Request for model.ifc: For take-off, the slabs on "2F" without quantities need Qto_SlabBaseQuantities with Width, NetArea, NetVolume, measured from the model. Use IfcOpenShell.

First a look at what the model holds.

```python
import ifcopenshell
import ifcopenshell.util.element
import ifcopenshell.util.unit

model = ifcopenshell.open("model.ifc")
print(model.schema)
for unit_type in ("LENGTHUNIT", "AREAUNIT", "VOLUMEUNIT"):
    print(unit_type, ifcopenshell.util.unit.calculate_unit_scale(model, unit_type))
storey = next(s for s in model.by_type("IfcBuildingStorey") if s.Name == "2F")
slabs = [e for e in ifcopenshell.util.element.get_decomposition(storey) if e.is_a("IfcSlab")]
for e in sorted(slabs, key=lambda e: e.id()):
    print(e.id(), e.is_a(), e.Name, list(ifcopenshell.util.element.get_psets(e, qtos_only=True)), sep=" | ")
```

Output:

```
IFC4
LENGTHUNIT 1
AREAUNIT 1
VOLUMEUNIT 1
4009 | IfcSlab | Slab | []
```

```python
import ifcopenshell
import ifcopenshell.api.pset
import ifcopenshell.geom
import ifcopenshell.util.element
import ifcopenshell.util.shape
import ifcopenshell.util.unit

model = ifcopenshell.open("model.ifc")
unit_scale = ifcopenshell.util.unit.calculate_unit_scale(model)
area_scale = ifcopenshell.util.unit.calculate_unit_scale(model, "AREAUNIT")
volume_scale = ifcopenshell.util.unit.calculate_unit_scale(model, "VOLUMEUNIT")
settings = ifcopenshell.geom.settings()

storey = next(s for s in model.by_type("IfcBuildingStorey") if s.Name == "2F")
slabs = [e for e in ifcopenshell.util.element.get_decomposition(storey) if e.is_a("IfcSlab")]

for e in sorted(slabs, key=lambda e: e.id()):
    if ifcopenshell.util.element.get_psets(e, qtos_only=True, should_inherit=False):
        continue
    # Geometry comes back in metres, in the element's own axes.
    shape = ifcopenshell.geom.create_shape(settings, e)
    values = {
        "Width": ifcopenshell.util.shape.get_z(shape.geometry) / unit_scale,
        "NetArea": ifcopenshell.util.shape.get_footprint_area(shape.geometry) / area_scale,
        "NetVolume": ifcopenshell.util.shape.get_volume(shape.geometry) / volume_scale,
    }
    qto = ifcopenshell.api.pset.add_qto(model, product=e, name="Qto_SlabBaseQuantities")
    ifcopenshell.api.pset.edit_qto(model, qto=qto, properties=values)
    print(e.id(), {k: round(v, 3) for k, v in values.items()})

model.write("model-out.ifc")
```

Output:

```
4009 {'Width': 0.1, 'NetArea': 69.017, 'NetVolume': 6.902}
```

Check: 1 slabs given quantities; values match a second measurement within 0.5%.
